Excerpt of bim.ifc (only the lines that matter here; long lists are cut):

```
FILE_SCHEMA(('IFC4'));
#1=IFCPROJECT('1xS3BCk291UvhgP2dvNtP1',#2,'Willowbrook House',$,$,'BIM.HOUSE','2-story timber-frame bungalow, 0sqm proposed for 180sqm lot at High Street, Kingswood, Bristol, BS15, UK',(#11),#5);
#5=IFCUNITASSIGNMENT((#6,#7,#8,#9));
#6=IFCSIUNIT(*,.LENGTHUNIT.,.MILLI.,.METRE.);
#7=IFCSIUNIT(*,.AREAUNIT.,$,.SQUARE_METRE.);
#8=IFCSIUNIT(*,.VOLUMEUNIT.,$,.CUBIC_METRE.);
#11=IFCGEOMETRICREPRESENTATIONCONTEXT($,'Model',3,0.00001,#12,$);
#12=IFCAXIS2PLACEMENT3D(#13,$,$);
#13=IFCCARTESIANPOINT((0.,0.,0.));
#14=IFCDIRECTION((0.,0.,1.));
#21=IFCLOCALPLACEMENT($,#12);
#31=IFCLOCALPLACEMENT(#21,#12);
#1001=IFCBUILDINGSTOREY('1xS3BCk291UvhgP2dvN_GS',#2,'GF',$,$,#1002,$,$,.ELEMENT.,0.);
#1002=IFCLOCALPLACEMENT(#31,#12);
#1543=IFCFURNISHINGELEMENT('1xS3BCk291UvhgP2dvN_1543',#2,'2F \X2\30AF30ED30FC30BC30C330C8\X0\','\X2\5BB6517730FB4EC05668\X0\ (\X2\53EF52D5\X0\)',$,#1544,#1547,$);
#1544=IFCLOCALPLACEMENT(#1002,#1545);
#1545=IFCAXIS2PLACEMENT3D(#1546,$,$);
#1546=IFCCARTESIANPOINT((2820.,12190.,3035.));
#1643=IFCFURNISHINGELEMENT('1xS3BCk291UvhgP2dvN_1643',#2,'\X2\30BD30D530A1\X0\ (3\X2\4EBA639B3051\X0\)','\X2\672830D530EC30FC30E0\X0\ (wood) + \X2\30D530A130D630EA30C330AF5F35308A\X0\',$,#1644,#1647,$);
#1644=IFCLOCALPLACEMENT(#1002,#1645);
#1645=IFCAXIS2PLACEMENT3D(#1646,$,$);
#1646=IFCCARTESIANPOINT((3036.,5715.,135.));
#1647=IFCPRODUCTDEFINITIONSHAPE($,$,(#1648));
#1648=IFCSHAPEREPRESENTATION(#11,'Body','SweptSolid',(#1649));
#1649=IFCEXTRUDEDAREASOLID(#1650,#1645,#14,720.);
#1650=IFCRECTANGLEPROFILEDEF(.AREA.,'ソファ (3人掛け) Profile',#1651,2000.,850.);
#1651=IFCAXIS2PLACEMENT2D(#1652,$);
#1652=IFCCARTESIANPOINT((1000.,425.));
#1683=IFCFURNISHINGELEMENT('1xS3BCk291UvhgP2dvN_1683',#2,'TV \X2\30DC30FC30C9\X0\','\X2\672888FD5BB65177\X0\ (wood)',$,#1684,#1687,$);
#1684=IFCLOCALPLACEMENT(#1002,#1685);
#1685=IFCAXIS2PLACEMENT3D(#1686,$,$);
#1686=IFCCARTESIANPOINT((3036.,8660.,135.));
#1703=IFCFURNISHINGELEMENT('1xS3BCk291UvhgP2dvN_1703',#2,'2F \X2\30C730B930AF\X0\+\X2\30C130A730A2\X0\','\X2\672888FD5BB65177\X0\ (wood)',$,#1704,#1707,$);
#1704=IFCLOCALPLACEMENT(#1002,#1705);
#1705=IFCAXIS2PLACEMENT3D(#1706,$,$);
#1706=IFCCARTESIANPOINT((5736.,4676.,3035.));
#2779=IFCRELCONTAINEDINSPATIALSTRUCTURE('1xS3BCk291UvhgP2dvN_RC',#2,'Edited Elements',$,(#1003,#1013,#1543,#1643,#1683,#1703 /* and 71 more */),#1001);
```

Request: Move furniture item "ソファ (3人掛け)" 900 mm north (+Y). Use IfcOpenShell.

```python
import ifcopenshell
import ifcopenshell.api.geometry
import ifcopenshell.util.placement
import ifcopenshell.util.unit

model = ifcopenshell.open("bim.ifc")
unit_scale = ifcopenshell.util.unit.calculate_unit_scale(model)

item = model.by_guid("1xS3BCk291UvhgP2dvN_1643")
matrix = ifcopenshell.util.placement.get_local_placement(item.ObjectPlacement)
matrix[1, 3] += 0.9 / unit_scale
ifcopenshell.api.geometry.edit_object_placement(model, product=item, matrix=matrix, is_si=False)

print(ifcopenshell.util.placement.get_local_placement(item.ObjectPlacement).round(3) + 0.0)

model.write("bim_edited.ifc")
```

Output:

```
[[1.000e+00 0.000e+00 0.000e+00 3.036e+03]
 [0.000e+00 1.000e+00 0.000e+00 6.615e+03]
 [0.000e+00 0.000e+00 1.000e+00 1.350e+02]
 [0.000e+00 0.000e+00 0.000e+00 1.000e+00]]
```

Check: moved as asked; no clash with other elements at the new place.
